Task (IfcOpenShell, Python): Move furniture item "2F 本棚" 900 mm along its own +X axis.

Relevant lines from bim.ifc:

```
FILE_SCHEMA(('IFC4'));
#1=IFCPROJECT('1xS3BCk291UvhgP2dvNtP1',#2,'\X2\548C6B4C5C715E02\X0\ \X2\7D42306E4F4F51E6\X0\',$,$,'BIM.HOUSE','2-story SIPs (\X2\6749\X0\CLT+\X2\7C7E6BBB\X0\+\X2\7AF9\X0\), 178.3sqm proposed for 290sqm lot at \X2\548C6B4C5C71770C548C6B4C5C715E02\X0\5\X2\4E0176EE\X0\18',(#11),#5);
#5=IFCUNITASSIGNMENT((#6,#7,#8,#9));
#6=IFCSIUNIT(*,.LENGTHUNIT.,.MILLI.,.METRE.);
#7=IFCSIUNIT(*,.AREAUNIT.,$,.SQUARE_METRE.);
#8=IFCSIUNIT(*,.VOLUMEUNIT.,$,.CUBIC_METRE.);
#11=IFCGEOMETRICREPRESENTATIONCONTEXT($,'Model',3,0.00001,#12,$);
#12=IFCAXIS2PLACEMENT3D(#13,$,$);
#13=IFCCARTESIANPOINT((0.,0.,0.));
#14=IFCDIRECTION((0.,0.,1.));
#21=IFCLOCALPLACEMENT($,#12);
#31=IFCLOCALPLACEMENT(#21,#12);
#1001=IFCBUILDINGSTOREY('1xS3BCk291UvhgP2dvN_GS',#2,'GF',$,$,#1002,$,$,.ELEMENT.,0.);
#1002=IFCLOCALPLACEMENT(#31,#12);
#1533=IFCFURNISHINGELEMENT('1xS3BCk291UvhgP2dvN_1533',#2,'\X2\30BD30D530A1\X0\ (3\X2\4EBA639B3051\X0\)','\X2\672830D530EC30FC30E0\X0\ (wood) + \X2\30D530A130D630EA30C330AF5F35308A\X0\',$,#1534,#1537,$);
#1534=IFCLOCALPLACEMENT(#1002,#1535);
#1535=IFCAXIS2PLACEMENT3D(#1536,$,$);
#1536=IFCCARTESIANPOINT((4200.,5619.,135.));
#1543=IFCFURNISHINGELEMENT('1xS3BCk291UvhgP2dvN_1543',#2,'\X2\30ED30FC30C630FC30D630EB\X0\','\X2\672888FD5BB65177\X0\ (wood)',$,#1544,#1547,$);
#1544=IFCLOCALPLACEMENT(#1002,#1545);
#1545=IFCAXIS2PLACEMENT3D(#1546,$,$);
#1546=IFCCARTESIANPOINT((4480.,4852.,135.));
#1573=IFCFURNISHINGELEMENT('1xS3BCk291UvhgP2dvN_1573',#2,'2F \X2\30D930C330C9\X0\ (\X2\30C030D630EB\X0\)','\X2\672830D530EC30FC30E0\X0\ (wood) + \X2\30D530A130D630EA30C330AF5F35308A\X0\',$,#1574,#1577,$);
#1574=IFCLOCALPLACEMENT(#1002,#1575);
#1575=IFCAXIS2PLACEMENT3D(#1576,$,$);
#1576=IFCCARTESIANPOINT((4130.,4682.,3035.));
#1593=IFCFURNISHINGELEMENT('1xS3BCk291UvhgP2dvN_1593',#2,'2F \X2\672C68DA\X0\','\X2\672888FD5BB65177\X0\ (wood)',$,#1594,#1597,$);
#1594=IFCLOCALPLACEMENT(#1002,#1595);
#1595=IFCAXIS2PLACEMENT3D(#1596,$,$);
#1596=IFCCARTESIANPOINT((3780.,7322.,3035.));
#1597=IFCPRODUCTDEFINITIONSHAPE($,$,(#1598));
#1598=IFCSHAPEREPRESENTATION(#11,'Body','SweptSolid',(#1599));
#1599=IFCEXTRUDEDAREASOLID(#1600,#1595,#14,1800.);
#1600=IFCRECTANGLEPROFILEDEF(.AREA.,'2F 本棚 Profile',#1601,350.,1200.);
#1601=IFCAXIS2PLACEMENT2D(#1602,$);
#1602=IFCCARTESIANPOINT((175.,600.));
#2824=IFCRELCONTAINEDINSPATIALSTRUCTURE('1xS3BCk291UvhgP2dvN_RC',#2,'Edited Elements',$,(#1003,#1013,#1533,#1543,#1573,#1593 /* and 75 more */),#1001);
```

```python
import ifcopenshell
import ifcopenshell.api.geometry
import ifcopenshell.util.placement

model = ifcopenshell.open("bim.ifc")

item = model.by_guid("1xS3BCk291UvhgP2dvN_1593")
matrix = ifcopenshell.util.placement.get_local_placement(item.ObjectPlacement)
matrix[:3, 3] += matrix[:3, 0] * 900.0
ifcopenshell.api.geometry.edit_object_placement(model, product=item, matrix=matrix, is_si=False)

print(ifcopenshell.util.placement.get_local_placement(item.ObjectPlacement).round(3) + 0.0)

model.write("bim_edited.ifc")
```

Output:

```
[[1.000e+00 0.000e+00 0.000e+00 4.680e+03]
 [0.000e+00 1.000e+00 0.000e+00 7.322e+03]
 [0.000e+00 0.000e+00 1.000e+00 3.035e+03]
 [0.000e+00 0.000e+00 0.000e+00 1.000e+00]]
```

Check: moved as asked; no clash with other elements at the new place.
